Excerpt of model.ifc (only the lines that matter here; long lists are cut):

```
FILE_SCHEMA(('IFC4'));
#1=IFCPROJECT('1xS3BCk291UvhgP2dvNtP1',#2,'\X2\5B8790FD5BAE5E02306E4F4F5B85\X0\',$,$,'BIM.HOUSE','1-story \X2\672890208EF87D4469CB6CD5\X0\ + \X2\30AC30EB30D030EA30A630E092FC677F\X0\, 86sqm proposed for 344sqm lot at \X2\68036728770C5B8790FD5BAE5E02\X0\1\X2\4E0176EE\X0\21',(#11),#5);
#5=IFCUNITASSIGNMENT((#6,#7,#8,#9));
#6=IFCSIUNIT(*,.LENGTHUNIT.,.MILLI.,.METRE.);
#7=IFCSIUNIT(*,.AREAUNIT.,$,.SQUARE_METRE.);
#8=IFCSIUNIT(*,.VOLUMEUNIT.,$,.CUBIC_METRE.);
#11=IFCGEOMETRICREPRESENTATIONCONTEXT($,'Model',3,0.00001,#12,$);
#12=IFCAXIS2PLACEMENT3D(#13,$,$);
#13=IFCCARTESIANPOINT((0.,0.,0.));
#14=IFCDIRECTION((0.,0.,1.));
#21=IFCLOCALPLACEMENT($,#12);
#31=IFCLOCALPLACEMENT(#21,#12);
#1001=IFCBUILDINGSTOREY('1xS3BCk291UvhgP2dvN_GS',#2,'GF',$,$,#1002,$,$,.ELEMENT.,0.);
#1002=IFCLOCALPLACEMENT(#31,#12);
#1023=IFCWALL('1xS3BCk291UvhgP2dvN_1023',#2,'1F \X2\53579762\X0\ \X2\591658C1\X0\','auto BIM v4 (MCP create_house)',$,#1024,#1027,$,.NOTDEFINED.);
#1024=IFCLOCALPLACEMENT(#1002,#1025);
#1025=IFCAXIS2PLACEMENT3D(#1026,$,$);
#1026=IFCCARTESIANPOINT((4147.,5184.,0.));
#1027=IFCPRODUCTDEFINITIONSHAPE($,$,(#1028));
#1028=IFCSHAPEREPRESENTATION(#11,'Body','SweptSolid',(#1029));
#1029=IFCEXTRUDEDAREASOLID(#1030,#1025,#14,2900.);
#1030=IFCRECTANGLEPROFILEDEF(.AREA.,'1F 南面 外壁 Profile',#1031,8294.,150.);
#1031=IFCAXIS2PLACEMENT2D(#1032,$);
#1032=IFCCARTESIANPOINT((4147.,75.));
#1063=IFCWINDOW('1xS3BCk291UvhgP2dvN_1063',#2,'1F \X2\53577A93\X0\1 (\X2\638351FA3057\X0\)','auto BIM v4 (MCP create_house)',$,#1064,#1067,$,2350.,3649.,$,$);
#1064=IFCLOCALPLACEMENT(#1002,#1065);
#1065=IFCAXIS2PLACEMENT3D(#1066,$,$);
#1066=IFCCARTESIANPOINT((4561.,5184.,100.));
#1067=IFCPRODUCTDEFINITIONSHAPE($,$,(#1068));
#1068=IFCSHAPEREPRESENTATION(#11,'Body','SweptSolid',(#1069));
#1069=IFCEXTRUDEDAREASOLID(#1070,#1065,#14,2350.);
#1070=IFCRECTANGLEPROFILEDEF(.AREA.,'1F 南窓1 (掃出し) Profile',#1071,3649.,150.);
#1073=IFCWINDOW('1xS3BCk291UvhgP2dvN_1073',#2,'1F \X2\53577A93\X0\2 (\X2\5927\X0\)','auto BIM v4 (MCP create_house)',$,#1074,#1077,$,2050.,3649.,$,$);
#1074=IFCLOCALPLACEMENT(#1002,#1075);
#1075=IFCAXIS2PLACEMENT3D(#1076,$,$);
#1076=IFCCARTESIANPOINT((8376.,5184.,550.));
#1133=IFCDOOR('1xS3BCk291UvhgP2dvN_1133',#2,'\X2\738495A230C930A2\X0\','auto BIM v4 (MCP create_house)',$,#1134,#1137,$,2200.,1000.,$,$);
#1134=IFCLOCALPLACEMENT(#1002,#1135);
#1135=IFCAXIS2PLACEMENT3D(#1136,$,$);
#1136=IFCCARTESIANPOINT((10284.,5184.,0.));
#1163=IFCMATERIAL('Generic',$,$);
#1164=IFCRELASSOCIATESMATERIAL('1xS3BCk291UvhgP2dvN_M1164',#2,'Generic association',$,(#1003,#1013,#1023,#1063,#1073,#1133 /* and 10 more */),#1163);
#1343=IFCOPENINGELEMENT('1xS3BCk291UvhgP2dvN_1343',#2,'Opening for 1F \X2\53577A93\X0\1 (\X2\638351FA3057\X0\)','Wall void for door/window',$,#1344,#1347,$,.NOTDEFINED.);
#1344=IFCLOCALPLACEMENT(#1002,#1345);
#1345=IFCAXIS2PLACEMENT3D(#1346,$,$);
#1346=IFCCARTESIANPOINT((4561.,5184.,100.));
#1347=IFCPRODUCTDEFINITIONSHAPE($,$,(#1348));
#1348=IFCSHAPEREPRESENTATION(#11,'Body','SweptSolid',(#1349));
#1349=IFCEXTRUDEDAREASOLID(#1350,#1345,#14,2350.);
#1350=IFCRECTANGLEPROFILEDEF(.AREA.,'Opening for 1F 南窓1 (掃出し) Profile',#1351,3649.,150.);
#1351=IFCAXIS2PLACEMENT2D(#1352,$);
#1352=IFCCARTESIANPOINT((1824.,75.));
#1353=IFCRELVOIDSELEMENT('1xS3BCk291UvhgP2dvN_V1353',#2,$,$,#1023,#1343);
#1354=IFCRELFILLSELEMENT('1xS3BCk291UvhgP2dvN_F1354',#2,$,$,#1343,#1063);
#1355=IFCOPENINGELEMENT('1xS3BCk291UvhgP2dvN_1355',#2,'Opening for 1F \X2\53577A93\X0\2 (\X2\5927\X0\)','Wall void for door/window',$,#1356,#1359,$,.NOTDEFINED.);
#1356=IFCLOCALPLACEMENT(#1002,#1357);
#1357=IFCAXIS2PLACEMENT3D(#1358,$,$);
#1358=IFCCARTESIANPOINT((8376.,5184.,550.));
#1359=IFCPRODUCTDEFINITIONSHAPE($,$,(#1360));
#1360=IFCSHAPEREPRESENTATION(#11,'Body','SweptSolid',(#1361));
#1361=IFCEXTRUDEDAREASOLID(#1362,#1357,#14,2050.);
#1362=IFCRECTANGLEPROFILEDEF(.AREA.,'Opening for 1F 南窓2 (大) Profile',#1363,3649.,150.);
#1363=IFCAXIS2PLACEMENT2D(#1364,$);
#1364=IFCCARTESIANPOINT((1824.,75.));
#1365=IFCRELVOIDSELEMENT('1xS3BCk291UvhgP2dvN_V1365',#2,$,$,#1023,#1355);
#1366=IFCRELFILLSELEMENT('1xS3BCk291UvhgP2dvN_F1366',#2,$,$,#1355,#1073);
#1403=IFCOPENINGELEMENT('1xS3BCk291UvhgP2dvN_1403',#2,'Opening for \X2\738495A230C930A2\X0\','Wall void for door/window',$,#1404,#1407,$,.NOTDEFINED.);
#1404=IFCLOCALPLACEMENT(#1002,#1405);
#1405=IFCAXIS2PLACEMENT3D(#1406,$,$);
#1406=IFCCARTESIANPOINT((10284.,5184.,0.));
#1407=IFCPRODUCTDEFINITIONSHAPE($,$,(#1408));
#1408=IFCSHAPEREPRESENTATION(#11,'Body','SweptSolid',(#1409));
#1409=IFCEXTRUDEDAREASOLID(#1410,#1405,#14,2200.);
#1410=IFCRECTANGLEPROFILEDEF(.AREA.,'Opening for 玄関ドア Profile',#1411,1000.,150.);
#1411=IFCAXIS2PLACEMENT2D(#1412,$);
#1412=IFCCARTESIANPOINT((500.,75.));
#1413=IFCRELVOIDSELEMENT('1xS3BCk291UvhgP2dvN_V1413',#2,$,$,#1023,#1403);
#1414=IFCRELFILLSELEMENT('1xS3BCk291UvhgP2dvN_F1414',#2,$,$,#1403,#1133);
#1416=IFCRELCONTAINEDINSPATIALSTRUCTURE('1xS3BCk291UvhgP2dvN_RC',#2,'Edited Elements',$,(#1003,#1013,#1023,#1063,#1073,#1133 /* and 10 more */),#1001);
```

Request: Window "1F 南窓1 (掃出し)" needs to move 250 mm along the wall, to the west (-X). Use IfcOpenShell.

```python
import ifcopenshell
import ifcopenshell.api.geometry
import ifcopenshell.util.placement
import ifcopenshell.util.unit

model = ifcopenshell.open("model.ifc")
unit_scale = ifcopenshell.util.unit.calculate_unit_scale(model)

window = model.by_guid("1xS3BCk291UvhgP2dvN_1063")
opening = window.FillsVoids[0].RelatingOpeningElement
wall = opening.VoidsElements[0].RelatingBuildingElement

wall_matrix = ifcopenshell.util.placement.get_local_placement(wall.ObjectPlacement)
shift = wall_matrix[:3, 0] * -0.25 / unit_scale
before = ifcopenshell.util.placement.get_local_placement(window.ObjectPlacement)[:3, 3].copy()

# The window is not placed relative to its opening, so move both.
for product in (opening, window):
    matrix = ifcopenshell.util.placement.get_local_placement(product.ObjectPlacement)
    matrix[:3, 3] += shift
    ifcopenshell.api.geometry.edit_object_placement(model, product=product, matrix=matrix, is_si=False)

after = ifcopenshell.util.placement.get_local_placement(window.ObjectPlacement)[:3, 3]
print("window moved by", (after - before).round(3) + 0.0)

model.write("model_edited.ifc")
```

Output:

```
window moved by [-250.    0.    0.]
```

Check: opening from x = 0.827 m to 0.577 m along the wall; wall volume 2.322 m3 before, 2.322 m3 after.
